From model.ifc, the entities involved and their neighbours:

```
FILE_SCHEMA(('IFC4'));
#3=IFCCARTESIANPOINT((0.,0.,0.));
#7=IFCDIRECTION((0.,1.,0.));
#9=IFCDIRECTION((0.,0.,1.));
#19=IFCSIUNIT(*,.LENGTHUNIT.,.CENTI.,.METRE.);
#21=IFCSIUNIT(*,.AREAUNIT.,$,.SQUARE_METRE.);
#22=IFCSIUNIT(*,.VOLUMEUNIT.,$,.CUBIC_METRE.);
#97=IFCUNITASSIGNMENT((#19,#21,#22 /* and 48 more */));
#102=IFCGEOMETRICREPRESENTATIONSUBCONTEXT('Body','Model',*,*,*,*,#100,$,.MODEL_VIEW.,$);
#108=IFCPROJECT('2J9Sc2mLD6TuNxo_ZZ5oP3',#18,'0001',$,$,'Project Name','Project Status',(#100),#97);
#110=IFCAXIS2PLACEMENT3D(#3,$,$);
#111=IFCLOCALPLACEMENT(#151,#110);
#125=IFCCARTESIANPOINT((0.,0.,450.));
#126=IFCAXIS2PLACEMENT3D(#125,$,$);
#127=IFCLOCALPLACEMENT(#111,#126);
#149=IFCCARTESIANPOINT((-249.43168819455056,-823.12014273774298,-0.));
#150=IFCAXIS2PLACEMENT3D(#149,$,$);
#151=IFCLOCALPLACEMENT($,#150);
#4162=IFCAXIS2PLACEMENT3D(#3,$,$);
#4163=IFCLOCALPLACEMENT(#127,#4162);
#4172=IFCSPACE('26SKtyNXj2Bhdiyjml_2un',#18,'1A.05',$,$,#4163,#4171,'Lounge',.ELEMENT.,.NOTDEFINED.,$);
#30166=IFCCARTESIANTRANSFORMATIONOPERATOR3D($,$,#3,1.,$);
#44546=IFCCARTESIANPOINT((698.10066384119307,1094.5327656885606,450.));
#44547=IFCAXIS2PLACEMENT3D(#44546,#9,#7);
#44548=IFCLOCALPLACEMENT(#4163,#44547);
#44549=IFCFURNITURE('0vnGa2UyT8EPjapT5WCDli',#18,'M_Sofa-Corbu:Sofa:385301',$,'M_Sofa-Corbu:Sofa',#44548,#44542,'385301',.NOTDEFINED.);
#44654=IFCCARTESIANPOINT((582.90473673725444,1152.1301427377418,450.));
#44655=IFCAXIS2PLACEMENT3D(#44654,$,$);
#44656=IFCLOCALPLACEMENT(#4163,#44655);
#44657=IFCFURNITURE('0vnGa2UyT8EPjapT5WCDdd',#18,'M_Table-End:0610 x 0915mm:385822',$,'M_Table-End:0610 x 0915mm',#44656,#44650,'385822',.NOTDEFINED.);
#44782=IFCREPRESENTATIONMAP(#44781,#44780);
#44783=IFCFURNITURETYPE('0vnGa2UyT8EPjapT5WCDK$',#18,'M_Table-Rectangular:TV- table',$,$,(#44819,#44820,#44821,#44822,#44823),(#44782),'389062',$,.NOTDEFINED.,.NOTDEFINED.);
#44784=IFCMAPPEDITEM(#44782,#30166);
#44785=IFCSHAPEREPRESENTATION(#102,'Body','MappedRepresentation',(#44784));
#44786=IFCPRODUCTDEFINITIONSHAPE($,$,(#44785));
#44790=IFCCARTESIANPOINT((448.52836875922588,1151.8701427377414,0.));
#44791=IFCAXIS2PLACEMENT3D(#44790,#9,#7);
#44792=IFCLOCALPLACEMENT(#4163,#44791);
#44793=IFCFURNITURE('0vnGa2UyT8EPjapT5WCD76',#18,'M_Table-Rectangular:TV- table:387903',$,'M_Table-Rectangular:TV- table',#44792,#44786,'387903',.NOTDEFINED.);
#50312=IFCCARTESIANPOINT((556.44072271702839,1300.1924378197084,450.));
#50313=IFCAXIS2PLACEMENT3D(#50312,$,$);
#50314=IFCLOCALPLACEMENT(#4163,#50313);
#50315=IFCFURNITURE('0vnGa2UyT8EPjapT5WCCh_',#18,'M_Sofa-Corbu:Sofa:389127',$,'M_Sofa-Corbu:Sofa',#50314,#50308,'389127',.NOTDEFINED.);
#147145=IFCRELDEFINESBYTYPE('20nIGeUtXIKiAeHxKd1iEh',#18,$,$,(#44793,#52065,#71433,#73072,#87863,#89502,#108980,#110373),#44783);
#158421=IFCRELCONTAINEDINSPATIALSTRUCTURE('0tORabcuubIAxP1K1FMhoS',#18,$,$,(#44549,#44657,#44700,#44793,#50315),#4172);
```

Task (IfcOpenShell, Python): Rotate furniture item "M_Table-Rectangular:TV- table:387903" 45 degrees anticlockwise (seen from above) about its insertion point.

```python
import ifcopenshell
import ifcopenshell.api.geometry
import ifcopenshell.util.placement

model = ifcopenshell.open("model.ifc")

item = model.by_id(44793)
matrix = ifcopenshell.util.placement.get_local_placement(item.ObjectPlacement)
matrix = matrix @ ifcopenshell.util.placement.rotation(45, "Z")
ifcopenshell.api.geometry.edit_object_placement(model, product=item, matrix=matrix, is_si=False)

print(ifcopenshell.util.placement.get_local_placement(item.ObjectPlacement).round(3) + 0.0)

model.write("model_updated.ifc")
```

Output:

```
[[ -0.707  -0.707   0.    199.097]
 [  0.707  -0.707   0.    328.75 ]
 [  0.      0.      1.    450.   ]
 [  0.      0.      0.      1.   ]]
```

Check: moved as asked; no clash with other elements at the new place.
